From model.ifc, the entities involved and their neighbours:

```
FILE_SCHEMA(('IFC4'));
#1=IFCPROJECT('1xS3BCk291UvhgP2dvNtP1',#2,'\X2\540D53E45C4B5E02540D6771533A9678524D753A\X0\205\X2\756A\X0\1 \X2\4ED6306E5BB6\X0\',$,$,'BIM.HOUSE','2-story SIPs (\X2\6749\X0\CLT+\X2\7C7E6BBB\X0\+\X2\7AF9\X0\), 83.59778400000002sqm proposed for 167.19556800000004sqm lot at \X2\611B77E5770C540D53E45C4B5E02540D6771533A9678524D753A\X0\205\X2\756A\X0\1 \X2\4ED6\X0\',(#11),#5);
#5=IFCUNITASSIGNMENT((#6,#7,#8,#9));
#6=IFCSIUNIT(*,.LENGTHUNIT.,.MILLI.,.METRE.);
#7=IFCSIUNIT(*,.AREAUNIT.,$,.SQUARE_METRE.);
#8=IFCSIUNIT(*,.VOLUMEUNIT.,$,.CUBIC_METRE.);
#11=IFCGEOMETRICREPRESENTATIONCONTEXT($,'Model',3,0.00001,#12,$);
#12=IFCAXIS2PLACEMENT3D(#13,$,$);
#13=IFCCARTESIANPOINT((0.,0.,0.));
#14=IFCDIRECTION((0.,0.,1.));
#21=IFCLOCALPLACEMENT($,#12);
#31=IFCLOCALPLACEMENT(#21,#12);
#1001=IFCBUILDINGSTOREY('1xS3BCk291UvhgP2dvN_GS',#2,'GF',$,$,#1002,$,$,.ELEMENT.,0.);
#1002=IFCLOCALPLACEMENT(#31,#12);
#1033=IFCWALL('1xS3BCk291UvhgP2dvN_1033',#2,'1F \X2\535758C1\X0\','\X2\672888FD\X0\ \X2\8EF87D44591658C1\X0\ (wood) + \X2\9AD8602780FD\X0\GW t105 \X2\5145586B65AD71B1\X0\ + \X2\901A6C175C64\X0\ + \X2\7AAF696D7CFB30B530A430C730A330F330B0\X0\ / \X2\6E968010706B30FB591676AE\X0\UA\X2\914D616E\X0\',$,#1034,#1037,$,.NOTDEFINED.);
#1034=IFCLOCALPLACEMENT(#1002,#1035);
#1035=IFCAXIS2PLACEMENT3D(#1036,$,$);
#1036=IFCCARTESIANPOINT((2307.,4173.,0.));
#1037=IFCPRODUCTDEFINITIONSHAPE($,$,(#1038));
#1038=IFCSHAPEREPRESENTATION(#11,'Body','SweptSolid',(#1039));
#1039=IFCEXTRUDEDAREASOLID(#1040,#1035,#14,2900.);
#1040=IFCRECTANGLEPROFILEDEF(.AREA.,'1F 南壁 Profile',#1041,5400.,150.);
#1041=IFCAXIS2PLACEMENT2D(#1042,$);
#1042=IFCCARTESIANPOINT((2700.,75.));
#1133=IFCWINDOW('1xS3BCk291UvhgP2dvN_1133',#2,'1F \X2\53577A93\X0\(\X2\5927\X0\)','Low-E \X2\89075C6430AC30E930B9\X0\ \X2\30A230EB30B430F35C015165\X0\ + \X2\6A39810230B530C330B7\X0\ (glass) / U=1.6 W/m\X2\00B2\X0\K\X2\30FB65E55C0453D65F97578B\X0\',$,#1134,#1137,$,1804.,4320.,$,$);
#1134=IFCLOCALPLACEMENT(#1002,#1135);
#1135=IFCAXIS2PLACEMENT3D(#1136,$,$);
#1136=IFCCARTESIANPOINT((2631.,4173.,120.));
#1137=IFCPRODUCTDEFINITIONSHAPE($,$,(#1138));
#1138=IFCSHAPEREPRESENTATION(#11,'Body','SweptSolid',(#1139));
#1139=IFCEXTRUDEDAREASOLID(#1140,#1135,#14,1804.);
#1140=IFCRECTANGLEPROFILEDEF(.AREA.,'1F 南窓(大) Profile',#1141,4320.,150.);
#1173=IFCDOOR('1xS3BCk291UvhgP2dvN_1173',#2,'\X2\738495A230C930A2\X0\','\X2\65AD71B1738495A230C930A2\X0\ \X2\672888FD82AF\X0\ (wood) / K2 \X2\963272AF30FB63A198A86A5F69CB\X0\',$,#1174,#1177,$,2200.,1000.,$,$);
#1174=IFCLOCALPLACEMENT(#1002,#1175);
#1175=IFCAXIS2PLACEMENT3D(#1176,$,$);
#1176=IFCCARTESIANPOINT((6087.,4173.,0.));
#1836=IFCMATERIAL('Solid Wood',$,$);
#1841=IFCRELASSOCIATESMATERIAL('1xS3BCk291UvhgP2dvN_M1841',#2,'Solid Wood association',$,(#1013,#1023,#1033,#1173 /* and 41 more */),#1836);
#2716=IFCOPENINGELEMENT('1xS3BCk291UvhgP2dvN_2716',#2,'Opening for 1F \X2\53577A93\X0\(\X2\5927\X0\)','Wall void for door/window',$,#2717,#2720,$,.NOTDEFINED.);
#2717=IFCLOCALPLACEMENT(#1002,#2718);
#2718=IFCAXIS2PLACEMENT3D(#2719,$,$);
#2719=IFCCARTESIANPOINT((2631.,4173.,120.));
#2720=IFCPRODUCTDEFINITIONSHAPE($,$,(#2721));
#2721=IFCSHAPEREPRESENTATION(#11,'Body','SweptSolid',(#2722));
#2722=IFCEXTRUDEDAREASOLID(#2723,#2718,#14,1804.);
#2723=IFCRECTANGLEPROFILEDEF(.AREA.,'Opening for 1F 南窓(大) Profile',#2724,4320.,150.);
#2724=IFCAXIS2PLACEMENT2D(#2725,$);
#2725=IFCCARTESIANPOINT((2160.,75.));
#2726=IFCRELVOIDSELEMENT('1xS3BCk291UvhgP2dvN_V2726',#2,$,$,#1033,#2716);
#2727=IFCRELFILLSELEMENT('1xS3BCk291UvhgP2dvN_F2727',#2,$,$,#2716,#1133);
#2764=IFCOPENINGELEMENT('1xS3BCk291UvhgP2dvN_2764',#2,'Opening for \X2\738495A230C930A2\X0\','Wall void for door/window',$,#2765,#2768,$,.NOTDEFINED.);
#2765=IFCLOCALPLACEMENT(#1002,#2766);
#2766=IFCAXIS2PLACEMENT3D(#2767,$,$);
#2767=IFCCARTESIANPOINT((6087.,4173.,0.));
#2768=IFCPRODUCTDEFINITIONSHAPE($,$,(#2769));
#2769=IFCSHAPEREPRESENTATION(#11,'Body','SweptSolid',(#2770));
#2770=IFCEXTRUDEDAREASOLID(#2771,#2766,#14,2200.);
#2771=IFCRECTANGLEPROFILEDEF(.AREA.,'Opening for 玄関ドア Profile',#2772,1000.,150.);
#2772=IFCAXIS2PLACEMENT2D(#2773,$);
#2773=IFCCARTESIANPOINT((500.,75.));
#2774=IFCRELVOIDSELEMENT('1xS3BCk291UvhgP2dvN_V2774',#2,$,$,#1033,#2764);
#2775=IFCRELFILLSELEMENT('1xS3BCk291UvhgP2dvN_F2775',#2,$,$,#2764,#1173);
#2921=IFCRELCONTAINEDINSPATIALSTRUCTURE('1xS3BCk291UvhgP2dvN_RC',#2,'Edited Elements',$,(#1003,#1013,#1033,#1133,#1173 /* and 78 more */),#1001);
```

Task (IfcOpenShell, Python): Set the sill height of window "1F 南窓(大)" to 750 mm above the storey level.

```python
import numpy as np
import ifcopenshell
import ifcopenshell.api.geometry
import ifcopenshell.geom
import ifcopenshell.util.element
import ifcopenshell.util.placement
import ifcopenshell.util.shape
import ifcopenshell.util.unit

model = ifcopenshell.open("model.ifc")
unit_scale = ifcopenshell.util.unit.calculate_unit_scale(model)

window = model.by_guid("1xS3BCk291UvhgP2dvN_1133")
opening = window.FillsVoids[0].RelatingOpeningElement
storey = ifcopenshell.util.element.get_container(window, ifc_class="IfcBuildingStorey")
level = ifcopenshell.util.placement.get_local_placement(storey.ObjectPlacement)[2, 3]

# The opening's origin need not be at the sill, so measure its lowest point.
shape = ifcopenshell.geom.create_shape(ifcopenshell.geom.settings(), opening)
bottom = ifcopenshell.util.shape.get_shape_bottom_elevation(shape, shape.geometry) / unit_scale
dz = level + 0.75 / unit_scale - bottom

shift = np.array([0.0, 0.0, dz])
# The window is not placed relative to its opening, so move both.
for product in (opening, window):
    matrix = ifcopenshell.util.placement.get_local_placement(product.ObjectPlacement)
    matrix[:3, 3] += shift
    ifcopenshell.api.geometry.edit_object_placement(model, product=product, matrix=matrix, is_si=False)

print(f"moved by {dz * unit_scale:+.3f} m")

model.write("model_v2.ifc")
```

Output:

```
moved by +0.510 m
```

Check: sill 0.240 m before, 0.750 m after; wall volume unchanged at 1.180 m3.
